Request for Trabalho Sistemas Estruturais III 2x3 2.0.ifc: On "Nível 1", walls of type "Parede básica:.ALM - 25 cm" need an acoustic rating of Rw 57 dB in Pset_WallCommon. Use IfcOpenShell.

First a look at what the model holds.

```python
import ifcopenshell
import ifcopenshell.util.element

model = ifcopenshell.open("Trabalho Sistemas Estruturais III 2x3 2.0.ifc")
print(model.schema)
storey = next(s for s in model.by_type("IfcBuildingStorey") if s.Name == "Nível 1")
walls = [e for e in ifcopenshell.util.element.get_decomposition(storey) if e.is_a("IfcWall")]
seen = {}
for e in walls:
    element_type = ifcopenshell.util.element.get_type(e)
    key = (element_type.Name if element_type != e and element_type else None, ifcopenshell.util.element.get_pset(e, "Pset_WallCommon", "AcousticRating"))
    seen[key] = seen.get(key, 0) + 1
for (name, value), count in sorted(seen.items(), key=str):
    print(count, "x", name, "|", value)
```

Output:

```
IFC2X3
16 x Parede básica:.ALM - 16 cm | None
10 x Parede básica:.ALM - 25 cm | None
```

```python
import ifcopenshell
import ifcopenshell.api.pset
import ifcopenshell.util.element

model = ifcopenshell.open("Trabalho Sistemas Estruturais III 2x3 2.0.ifc")

storey = next(s for s in model.by_type("IfcBuildingStorey") if s.Name == "Nível 1")
walls = [e for e in ifcopenshell.util.element.get_decomposition(storey) if e.is_a("IfcWall")]

count = 0
for e in walls:
    element_type = ifcopenshell.util.element.get_type(e)
    if element_type in (None, e) or element_type.Name != "Parede básica:.ALM - 25 cm":
        continue
    # add_pset returns the element's existing set when there is one.
    pset = ifcopenshell.api.pset.add_pset(model, product=e, name="Pset_WallCommon")
    ifcopenshell.api.pset.edit_pset(model, pset=pset, properties={"AcousticRating": "Rw 57 dB"})
    count += 1

print(count, "walls updated")

model.write("Trabalho Sistemas Estruturais III 2x3 2.0-out.ifc")
```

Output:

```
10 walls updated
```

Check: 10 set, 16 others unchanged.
